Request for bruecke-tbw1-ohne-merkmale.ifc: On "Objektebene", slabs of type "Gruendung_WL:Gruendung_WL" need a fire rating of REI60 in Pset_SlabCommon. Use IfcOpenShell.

First a look at what the model holds.

```python
import ifcopenshell
import ifcopenshell.util.element

model = ifcopenshell.open("bruecke-tbw1-ohne-merkmale.ifc")
print(model.schema)
storey = next(s for s in model.by_type("IfcBuildingStorey") if s.Name == "Objektebene")
slabs = [e for e in ifcopenshell.util.element.get_decomposition(storey) if e.is_a("IfcSlab")]
seen = {}
for e in slabs:
    element_type = ifcopenshell.util.element.get_type(e)
    key = (element_type.Name if element_type != e and element_type else None, ifcopenshell.util.element.get_pset(e, "Pset_SlabCommon", "FireRating"))
    seen[key] = seen.get(key, 0) + 1
for (name, value), count in sorted(seen.items(), key=str):
    print(count, "x", name, "|", value)
```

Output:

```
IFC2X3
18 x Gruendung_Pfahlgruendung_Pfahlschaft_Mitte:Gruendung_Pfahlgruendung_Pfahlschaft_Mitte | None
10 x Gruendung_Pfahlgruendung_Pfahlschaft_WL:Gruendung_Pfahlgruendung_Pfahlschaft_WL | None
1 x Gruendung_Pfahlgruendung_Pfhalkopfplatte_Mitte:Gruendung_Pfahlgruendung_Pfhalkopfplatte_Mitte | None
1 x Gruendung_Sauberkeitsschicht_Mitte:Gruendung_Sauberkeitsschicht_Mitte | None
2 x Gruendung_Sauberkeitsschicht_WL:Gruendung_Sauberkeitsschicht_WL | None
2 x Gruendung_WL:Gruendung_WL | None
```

```python
import ifcopenshell
import ifcopenshell.api.pset
import ifcopenshell.util.element

model = ifcopenshell.open("bruecke-tbw1-ohne-merkmale.ifc")

storey = next(s for s in model.by_type("IfcBuildingStorey") if s.Name == "Objektebene")
slabs = [e for e in ifcopenshell.util.element.get_decomposition(storey) if e.is_a("IfcSlab")]

count = 0
for e in slabs:
    element_type = ifcopenshell.util.element.get_type(e)
    if element_type in (None, e) or element_type.Name != "Gruendung_WL:Gruendung_WL":
        continue
    # add_pset returns the element's existing set when there is one.
    pset = ifcopenshell.api.pset.add_pset(model, product=e, name="Pset_SlabCommon")
    ifcopenshell.api.pset.edit_pset(model, pset=pset, properties={"FireRating": "REI60"})
    count += 1

print(count, "slabs updated")

model.write("bruecke-tbw1-ohne-merkmale_rev.ifc")
```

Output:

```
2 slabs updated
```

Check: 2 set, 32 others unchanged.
